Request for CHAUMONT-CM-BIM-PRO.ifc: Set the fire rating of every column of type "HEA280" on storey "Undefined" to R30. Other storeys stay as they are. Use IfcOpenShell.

First a look at what the model holds.

```python
import ifcopenshell
import ifcopenshell.util.element

model = ifcopenshell.open("CHAUMONT-CM-BIM-PRO.ifc")
print(model.schema)
storey = next(s for s in model.by_type("IfcBuildingStorey") if s.Name == "Undefined")
columns = [e for e in ifcopenshell.util.element.get_decomposition(storey) if e.is_a("IfcColumn")]
seen = {}
for e in columns:
    element_type = ifcopenshell.util.element.get_type(e)
    key = (element_type.Name if element_type != e and element_type else None, ifcopenshell.util.element.get_pset(e, "Pset_ColumnCommon", "FireRating"))
    seen[key] = seen.get(key, 0) + 1
for (name, value), count in sorted(seen.items(), key=str):
    print(count, "x", name, "|", value)
```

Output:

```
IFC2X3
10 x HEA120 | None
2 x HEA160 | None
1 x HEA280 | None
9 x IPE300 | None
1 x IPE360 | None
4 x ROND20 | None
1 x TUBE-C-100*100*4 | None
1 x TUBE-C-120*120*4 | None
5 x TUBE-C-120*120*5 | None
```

```python
import ifcopenshell
import ifcopenshell.api.pset
import ifcopenshell.util.element

model = ifcopenshell.open("CHAUMONT-CM-BIM-PRO.ifc")

storey = next(s for s in model.by_type("IfcBuildingStorey") if s.Name == "Undefined")
columns = [e for e in ifcopenshell.util.element.get_decomposition(storey) if e.is_a("IfcColumn")]

count = 0
for e in columns:
    element_type = ifcopenshell.util.element.get_type(e)
    if element_type in (None, e) or element_type.Name != "HEA280":
        continue
    found = ifcopenshell.util.element.get_pset(e, "Pset_ColumnCommon", should_inherit=False)
    if found:
        pset = model.by_id(found["id"])
        if len(ifcopenshell.util.element.get_elements_by_pset(pset)) > 1:
            pset = ifcopenshell.api.pset.unshare_pset(model, products=[e], pset=pset)[0]
    else:
        pset = ifcopenshell.api.pset.add_pset(model, product=e, name="Pset_ColumnCommon")
    ifcopenshell.api.pset.edit_pset(model, pset=pset, properties={"FireRating": "R30"})
    count += 1

print(count, "columns updated")

model.write("CHAUMONT-CM-BIM-PRO_updated.ifc")
```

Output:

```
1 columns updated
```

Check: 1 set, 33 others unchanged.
